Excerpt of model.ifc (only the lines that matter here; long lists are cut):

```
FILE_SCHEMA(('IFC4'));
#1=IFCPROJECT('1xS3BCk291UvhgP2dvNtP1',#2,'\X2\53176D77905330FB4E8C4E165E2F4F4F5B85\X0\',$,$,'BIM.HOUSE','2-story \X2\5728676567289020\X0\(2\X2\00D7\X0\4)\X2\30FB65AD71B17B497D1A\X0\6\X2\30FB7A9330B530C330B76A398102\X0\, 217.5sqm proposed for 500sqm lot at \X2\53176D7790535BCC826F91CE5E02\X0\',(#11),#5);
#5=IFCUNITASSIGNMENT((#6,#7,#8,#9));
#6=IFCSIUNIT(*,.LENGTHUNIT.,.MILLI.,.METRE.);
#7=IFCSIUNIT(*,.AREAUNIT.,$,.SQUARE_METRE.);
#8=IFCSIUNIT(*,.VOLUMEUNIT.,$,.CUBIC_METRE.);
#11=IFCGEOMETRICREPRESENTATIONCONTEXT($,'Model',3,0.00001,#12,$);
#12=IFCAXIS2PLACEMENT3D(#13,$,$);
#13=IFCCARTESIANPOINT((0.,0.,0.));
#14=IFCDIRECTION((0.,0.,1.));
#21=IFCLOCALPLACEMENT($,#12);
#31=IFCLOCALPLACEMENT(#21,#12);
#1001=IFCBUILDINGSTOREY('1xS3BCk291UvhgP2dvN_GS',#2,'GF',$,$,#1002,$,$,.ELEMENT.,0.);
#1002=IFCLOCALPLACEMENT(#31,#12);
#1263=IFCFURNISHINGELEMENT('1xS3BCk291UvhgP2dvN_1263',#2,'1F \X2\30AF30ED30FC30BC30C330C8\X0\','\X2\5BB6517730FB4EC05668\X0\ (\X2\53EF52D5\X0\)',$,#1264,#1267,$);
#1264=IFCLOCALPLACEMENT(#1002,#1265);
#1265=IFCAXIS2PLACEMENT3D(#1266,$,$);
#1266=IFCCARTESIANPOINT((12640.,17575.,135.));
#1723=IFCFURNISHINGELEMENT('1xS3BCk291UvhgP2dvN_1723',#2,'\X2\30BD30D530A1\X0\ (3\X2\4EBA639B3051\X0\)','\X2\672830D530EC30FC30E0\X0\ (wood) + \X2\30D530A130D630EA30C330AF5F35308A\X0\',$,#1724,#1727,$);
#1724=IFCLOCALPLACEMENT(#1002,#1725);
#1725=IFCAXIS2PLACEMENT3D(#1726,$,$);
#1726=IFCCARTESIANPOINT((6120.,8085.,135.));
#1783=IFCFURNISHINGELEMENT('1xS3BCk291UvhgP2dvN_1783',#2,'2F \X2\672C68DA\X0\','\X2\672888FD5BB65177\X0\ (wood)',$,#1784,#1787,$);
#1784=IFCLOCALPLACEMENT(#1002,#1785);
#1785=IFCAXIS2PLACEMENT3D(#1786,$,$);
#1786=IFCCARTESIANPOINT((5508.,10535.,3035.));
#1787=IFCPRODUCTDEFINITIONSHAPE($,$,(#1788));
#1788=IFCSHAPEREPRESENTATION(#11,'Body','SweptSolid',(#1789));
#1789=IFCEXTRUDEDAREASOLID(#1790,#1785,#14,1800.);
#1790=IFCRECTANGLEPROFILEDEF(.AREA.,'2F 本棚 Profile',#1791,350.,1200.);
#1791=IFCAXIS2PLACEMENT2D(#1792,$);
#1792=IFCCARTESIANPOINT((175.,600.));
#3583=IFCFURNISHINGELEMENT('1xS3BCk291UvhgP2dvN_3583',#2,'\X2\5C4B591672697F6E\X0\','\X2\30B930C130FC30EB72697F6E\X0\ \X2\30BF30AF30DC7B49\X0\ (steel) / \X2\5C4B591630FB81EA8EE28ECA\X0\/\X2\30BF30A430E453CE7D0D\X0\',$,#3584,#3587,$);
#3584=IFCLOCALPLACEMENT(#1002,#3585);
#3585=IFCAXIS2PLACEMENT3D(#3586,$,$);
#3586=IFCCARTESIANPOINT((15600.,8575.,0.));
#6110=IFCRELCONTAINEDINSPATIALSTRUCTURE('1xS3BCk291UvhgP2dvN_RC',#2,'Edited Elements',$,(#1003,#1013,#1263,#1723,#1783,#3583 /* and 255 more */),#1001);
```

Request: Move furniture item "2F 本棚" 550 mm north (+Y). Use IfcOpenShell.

```python
import ifcopenshell
import ifcopenshell.api.geometry
import ifcopenshell.util.placement
import ifcopenshell.util.unit

model = ifcopenshell.open("model.ifc")
unit_scale = ifcopenshell.util.unit.calculate_unit_scale(model)

item = model.by_guid("1xS3BCk291UvhgP2dvN_1783")
matrix = ifcopenshell.util.placement.get_local_placement(item.ObjectPlacement)
matrix[1, 3] += 0.55 / unit_scale
ifcopenshell.api.geometry.edit_object_placement(model, product=item, matrix=matrix, is_si=False)

print(ifcopenshell.util.placement.get_local_placement(item.ObjectPlacement).round(3) + 0.0)

model.write("model_updated.ifc")
```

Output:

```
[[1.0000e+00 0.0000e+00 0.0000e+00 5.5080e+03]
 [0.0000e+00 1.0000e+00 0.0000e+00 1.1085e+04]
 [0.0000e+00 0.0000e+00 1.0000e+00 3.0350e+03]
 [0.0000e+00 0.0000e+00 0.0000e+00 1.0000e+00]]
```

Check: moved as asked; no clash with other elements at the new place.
